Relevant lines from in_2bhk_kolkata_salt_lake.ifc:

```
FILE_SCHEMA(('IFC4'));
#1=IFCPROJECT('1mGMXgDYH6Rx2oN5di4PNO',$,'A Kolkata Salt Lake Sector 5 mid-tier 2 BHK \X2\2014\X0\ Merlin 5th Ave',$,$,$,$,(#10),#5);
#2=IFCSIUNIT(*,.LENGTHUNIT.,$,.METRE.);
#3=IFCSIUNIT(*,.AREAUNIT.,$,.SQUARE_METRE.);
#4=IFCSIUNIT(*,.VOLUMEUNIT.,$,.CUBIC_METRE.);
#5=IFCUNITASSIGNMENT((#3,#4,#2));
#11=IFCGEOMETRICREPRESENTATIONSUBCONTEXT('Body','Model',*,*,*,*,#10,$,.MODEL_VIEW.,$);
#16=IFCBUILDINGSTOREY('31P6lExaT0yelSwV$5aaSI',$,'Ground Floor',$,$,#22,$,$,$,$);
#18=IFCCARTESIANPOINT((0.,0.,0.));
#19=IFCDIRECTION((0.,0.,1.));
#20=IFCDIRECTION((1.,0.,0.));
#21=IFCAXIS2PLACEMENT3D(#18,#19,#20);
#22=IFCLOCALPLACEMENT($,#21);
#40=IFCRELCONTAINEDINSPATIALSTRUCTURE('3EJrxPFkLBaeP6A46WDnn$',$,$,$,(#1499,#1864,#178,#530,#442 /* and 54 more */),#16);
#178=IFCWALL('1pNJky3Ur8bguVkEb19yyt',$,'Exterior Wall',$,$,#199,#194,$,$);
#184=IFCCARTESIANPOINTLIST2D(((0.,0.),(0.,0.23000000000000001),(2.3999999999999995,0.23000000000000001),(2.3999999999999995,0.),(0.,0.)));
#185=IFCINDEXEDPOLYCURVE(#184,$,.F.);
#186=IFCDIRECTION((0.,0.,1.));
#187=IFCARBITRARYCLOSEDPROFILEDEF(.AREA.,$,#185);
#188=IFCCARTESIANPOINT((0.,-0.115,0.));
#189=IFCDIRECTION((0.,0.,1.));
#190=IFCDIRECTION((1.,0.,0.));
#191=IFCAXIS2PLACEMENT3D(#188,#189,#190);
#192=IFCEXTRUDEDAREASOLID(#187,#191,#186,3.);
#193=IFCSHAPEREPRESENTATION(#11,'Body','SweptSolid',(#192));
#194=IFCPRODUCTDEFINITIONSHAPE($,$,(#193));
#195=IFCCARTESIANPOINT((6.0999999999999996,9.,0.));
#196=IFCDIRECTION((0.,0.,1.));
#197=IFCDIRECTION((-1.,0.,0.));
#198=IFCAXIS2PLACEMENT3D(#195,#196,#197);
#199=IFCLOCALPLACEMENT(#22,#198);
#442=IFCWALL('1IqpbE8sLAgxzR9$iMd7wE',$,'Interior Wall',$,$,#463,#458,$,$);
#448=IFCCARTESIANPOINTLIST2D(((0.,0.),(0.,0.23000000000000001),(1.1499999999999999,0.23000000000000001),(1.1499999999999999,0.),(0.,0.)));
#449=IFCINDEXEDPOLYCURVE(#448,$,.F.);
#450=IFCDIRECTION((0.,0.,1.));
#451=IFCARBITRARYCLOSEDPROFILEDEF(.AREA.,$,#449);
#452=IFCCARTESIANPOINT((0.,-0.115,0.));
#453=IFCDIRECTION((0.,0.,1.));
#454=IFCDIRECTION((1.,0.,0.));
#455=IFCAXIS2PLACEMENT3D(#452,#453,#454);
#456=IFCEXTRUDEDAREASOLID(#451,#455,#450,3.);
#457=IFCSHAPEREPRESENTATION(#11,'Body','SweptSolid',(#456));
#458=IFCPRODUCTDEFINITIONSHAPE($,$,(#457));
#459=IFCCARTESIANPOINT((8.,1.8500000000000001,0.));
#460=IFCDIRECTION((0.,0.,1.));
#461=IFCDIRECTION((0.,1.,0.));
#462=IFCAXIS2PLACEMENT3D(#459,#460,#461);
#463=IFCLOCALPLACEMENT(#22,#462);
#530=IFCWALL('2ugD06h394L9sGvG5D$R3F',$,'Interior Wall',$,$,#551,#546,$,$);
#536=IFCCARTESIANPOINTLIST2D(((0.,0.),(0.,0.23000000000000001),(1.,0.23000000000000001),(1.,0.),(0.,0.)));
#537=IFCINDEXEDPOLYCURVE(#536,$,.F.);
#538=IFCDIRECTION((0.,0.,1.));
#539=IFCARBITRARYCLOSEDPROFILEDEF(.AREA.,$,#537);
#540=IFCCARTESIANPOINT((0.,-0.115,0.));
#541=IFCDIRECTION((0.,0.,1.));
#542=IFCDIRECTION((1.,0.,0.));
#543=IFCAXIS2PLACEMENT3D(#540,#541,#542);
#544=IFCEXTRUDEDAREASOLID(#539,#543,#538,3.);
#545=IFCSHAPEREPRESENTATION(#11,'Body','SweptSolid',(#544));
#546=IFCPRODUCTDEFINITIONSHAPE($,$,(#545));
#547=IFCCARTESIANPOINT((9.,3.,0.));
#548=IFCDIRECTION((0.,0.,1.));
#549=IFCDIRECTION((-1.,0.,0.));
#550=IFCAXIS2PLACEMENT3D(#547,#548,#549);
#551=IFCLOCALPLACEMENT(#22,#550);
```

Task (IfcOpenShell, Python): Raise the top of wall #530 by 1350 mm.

```python
import ifcopenshell
import ifcopenshell.geom
import ifcopenshell.util.representation
import ifcopenshell.util.shape
import ifcopenshell.util.unit

model = ifcopenshell.open("in_2bhk_kolkata_salt_lake.ifc")
unit_scale = ifcopenshell.util.unit.calculate_unit_scale(model)
settings = ifcopenshell.geom.settings()


def volume(element):
    """Net volume in cubic metres, openings subtracted."""
    shape = ifcopenshell.geom.create_shape(settings, element)
    return ifcopenshell.util.shape.get_volume(shape.geometry)


wall = model.by_guid("2ugD06h394L9sGvG5D$R3F")
before = volume(wall)

body = ifcopenshell.util.representation.get_representation(wall, "Model", "Body")
solid = body.Items[0]
old_height = solid.Depth
solid.Depth += 1.35 / unit_scale
after = volume(wall)

print(f"height {old_height:g} -> {solid.Depth:g}, volume {before:.3f} -> {after:.3f} m3")

model.write("in_2bhk_kolkata_salt_lake_rev.ifc")
```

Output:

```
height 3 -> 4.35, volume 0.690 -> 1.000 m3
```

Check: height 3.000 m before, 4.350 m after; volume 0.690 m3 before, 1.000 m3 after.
